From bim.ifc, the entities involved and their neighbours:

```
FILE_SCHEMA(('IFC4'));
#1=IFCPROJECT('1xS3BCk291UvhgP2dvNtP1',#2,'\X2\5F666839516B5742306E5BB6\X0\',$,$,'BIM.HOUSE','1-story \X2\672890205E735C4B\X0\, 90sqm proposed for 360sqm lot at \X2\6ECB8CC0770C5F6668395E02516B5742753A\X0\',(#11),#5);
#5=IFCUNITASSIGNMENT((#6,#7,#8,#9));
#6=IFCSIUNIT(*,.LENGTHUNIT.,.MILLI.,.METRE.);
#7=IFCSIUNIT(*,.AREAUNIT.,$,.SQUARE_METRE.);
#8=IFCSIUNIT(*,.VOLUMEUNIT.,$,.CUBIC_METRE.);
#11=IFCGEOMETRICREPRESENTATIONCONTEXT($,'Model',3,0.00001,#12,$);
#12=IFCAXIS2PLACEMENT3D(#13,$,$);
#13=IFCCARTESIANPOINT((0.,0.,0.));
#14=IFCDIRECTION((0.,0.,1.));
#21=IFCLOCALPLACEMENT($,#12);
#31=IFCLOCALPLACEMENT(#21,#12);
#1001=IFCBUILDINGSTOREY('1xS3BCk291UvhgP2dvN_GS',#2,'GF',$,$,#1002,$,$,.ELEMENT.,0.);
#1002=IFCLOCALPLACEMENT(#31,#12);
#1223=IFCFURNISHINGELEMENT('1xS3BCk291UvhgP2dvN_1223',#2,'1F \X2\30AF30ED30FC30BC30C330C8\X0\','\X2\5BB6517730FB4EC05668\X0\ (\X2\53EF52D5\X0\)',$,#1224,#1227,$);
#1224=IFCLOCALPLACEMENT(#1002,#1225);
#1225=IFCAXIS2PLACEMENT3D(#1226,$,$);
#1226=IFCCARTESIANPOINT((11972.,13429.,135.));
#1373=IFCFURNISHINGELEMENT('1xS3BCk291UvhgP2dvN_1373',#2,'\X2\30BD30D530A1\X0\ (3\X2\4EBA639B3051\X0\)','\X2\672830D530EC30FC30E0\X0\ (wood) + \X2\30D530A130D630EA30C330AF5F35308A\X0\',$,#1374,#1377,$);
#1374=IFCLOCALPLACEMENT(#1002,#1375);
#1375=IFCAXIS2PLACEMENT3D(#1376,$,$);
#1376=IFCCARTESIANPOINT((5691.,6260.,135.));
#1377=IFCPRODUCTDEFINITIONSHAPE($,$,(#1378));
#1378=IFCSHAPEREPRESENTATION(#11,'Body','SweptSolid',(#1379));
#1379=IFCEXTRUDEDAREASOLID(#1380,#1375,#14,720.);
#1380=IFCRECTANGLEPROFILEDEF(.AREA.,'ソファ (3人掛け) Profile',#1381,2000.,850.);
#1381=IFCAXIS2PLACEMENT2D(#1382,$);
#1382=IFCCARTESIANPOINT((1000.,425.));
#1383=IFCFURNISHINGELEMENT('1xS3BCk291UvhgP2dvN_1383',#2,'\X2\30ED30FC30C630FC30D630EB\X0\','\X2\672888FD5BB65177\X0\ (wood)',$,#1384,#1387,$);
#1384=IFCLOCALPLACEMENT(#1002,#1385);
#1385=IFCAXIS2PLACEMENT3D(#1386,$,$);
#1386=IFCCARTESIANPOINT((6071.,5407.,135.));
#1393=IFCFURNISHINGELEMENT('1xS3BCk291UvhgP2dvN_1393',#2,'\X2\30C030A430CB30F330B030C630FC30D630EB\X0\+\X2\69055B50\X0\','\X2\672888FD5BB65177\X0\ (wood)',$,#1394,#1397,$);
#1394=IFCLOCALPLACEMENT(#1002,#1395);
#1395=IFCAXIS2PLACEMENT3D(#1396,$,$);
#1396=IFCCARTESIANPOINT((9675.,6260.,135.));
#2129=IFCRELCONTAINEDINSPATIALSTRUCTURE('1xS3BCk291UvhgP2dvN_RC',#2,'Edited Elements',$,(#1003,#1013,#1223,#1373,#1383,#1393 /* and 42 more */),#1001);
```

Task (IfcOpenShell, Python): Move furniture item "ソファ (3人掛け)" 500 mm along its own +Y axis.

```python
import ifcopenshell
import ifcopenshell.api.geometry
import ifcopenshell.util.placement
import ifcopenshell.util.unit

model = ifcopenshell.open("bim.ifc")
unit_scale = ifcopenshell.util.unit.calculate_unit_scale(model)

item = model.by_guid("1xS3BCk291UvhgP2dvN_1373")
matrix = ifcopenshell.util.placement.get_local_placement(item.ObjectPlacement)
matrix[:3, 3] += matrix[:3, 1] * 0.5 / unit_scale
ifcopenshell.api.geometry.edit_object_placement(model, product=item, matrix=matrix, is_si=False)

print(ifcopenshell.util.placement.get_local_placement(item.ObjectPlacement).round(3) + 0.0)

model.write("bim_updated.ifc")
```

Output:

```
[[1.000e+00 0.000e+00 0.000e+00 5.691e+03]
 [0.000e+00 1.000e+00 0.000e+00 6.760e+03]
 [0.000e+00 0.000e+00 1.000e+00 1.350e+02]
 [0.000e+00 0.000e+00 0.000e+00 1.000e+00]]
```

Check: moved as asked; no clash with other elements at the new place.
